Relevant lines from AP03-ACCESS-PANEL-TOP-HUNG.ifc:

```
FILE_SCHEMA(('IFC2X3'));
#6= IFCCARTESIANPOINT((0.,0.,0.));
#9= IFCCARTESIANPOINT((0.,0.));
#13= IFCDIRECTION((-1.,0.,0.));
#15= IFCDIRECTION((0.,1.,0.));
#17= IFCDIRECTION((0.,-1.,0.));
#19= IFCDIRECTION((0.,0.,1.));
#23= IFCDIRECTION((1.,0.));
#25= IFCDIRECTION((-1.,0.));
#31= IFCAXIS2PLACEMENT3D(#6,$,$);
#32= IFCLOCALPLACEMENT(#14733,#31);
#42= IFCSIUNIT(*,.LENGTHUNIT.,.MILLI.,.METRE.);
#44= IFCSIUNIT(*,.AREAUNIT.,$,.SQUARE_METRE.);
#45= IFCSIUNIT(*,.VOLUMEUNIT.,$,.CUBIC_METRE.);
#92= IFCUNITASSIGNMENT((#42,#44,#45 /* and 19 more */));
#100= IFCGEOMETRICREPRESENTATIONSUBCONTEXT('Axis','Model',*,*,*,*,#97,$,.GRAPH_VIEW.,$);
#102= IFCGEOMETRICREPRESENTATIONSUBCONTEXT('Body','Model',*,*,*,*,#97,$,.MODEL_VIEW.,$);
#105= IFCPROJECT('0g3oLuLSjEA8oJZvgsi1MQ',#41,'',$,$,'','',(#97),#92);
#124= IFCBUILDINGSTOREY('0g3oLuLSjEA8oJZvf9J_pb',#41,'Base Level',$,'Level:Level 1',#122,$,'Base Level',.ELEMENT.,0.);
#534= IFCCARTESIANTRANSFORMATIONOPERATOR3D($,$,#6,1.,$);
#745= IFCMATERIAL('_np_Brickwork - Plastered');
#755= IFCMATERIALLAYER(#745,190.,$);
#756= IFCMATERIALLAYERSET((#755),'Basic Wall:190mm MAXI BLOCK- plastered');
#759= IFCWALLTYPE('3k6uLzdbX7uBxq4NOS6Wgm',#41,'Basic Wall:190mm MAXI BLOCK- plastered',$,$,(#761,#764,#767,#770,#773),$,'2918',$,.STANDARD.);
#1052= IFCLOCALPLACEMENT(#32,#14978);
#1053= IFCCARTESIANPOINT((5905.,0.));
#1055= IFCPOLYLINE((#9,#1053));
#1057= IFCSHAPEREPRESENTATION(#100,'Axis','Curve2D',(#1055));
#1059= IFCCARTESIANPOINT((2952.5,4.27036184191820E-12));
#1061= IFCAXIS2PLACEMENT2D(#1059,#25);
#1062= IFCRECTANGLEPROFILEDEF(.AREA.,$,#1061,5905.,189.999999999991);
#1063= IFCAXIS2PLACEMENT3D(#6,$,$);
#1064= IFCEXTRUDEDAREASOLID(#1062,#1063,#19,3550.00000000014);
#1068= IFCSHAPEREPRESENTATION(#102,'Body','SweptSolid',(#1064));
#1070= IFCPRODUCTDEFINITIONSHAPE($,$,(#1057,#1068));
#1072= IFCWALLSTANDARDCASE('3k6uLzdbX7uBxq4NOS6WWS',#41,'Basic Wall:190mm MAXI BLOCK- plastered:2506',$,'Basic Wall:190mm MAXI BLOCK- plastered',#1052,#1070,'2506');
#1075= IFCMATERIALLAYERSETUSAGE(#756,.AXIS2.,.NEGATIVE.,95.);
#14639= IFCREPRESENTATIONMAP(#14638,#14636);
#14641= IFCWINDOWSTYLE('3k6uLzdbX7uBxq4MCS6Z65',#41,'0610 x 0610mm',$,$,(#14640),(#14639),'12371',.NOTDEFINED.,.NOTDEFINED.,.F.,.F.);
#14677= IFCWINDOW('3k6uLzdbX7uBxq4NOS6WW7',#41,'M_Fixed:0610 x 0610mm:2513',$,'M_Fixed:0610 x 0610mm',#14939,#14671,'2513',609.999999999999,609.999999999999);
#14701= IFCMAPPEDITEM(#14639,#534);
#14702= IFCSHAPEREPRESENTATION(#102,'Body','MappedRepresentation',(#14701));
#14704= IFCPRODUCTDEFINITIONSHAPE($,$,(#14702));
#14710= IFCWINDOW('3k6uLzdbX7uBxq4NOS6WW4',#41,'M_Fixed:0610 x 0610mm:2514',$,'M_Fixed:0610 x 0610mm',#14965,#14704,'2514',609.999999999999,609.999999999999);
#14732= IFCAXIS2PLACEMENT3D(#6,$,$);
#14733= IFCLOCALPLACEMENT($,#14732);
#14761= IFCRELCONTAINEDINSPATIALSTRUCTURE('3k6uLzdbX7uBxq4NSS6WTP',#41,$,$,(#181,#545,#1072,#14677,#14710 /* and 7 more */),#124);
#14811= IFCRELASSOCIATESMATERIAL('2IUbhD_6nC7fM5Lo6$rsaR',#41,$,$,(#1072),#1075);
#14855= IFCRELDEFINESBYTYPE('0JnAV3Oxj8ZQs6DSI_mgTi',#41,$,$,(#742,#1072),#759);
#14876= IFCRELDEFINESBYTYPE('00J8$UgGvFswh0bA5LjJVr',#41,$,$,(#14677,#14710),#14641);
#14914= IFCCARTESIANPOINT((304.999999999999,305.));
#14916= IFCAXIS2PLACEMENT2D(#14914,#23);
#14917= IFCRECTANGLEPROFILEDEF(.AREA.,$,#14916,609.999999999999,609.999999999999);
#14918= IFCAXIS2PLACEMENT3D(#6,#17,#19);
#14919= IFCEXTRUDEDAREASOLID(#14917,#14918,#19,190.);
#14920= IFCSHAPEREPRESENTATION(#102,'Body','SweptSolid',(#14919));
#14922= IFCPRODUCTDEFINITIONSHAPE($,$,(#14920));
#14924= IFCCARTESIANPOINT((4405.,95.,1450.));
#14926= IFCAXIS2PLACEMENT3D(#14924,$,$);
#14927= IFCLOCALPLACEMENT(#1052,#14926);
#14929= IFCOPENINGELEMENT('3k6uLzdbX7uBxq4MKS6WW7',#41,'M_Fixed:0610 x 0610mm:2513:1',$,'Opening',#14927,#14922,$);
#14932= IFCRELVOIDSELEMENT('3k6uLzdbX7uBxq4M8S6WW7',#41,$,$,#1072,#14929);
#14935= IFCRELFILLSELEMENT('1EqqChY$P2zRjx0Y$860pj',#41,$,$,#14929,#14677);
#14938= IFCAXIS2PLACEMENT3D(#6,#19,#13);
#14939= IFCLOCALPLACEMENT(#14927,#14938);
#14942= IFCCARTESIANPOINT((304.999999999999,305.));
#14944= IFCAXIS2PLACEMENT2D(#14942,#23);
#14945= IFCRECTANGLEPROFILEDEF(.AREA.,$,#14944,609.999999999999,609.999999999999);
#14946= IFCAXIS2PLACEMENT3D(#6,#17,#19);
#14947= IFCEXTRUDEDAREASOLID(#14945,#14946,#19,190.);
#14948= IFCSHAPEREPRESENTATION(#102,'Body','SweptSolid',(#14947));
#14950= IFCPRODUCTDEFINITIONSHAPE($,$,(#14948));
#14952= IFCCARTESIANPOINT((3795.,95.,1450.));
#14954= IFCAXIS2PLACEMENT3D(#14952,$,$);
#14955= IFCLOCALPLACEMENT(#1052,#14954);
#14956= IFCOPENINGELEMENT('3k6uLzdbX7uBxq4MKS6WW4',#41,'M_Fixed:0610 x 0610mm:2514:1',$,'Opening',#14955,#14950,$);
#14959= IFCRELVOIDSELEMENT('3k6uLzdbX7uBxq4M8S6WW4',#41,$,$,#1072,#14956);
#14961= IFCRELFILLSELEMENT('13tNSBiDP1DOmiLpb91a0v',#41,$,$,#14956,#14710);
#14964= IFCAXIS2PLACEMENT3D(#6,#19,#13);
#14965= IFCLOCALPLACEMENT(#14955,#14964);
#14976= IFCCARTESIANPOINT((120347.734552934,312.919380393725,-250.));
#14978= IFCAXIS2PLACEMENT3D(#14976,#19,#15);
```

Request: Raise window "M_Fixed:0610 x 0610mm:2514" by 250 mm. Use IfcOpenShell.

```python
import numpy as np
import ifcopenshell
import ifcopenshell.api.geometry
import ifcopenshell.util.placement
import ifcopenshell.util.unit

model = ifcopenshell.open("AP03-ACCESS-PANEL-TOP-HUNG.ifc")
unit_scale = ifcopenshell.util.unit.calculate_unit_scale(model)

window = model.by_guid("3k6uLzdbX7uBxq4NOS6WW4")
opening = window.FillsVoids[0].RelatingOpeningElement
dz = 0.25 / unit_scale

shift = np.array([0.0, 0.0, dz])
# The window is placed relative to its opening, so it follows when the opening moves.
matrix = ifcopenshell.util.placement.get_local_placement(opening.ObjectPlacement)
matrix[:3, 3] += shift
ifcopenshell.api.geometry.edit_object_placement(
    model, product=opening, matrix=matrix, is_si=False, should_transform_children=True
)

print(f"moved by {dz * unit_scale:+.3f} m")

model.write("AP03-ACCESS-PANEL-TOP-HUNG_v2.ifc")
```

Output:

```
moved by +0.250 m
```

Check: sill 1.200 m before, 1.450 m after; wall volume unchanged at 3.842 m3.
